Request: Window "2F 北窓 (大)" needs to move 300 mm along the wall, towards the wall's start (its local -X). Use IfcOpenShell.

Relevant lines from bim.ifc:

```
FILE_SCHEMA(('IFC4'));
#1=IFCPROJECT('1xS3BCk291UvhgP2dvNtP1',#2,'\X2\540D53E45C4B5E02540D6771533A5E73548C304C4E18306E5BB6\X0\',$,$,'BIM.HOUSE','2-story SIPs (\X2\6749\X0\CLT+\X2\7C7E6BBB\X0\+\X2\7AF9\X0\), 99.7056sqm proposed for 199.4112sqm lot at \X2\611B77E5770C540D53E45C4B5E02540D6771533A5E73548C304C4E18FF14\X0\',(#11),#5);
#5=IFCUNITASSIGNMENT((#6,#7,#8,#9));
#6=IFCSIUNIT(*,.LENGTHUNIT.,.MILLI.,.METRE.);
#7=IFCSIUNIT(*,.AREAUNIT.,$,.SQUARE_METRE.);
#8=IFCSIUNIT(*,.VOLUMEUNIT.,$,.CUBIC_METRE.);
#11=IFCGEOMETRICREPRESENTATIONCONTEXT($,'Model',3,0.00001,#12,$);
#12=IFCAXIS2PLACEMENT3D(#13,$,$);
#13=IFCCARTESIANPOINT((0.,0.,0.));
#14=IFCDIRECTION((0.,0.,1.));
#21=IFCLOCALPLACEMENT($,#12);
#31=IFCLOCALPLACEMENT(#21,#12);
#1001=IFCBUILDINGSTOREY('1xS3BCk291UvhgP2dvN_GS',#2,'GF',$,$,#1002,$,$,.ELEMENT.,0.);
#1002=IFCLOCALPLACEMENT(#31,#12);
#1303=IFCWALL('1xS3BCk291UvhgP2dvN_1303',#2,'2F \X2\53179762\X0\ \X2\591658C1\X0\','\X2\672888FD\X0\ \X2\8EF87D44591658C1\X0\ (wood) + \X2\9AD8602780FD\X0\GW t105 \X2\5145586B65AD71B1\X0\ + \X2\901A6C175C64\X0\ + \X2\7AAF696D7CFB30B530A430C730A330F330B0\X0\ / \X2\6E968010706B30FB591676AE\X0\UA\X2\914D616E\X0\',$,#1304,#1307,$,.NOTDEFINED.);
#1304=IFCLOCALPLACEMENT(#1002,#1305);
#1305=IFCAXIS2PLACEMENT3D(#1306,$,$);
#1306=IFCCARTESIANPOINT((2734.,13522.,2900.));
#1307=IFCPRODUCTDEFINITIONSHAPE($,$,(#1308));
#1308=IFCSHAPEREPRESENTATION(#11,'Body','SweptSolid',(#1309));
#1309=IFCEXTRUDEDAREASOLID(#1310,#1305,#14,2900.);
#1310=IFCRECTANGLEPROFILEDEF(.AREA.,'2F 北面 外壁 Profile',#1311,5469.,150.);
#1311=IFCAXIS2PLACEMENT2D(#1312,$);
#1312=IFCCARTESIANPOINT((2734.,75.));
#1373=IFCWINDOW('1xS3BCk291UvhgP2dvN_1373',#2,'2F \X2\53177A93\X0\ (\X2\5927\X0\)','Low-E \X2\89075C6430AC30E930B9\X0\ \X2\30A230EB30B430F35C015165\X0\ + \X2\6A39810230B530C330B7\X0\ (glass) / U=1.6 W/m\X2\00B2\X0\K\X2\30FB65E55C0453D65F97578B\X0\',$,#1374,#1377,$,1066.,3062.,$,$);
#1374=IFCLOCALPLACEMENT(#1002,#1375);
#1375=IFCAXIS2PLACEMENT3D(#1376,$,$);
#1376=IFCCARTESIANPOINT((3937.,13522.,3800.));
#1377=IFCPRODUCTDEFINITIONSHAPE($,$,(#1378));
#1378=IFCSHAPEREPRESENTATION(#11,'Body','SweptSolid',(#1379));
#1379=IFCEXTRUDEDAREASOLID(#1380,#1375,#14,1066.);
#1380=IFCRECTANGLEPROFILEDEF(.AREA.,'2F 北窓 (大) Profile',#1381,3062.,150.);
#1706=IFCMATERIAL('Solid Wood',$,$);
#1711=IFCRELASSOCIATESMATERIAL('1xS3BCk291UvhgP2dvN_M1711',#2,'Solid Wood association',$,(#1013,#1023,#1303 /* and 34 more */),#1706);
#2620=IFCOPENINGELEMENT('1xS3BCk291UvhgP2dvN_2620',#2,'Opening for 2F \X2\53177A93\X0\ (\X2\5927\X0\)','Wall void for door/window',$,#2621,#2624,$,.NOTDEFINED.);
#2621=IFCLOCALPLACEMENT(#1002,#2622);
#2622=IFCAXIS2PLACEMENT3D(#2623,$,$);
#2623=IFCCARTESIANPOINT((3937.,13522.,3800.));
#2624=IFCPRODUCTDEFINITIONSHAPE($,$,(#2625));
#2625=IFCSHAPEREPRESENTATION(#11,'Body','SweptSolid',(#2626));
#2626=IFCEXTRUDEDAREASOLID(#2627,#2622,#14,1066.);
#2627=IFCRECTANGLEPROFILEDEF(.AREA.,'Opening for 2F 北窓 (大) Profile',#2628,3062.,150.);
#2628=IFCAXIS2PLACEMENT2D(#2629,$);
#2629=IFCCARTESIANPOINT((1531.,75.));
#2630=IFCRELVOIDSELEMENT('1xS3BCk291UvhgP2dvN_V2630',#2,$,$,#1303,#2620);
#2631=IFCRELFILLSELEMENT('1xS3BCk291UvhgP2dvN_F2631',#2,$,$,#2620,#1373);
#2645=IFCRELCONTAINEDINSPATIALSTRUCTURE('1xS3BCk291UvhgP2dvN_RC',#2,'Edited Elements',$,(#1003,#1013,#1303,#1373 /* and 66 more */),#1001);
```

```python
import ifcopenshell
import ifcopenshell.api.geometry
import ifcopenshell.util.placement

model = ifcopenshell.open("bim.ifc")

window = model.by_id(1373)
opening = window.FillsVoids[0].RelatingOpeningElement
wall = opening.VoidsElements[0].RelatingBuildingElement

wall_matrix = ifcopenshell.util.placement.get_local_placement(wall.ObjectPlacement)
shift = wall_matrix[:3, 0] * -300.0
before = ifcopenshell.util.placement.get_local_placement(window.ObjectPlacement)[:3, 3].copy()

# The window is not placed relative to its opening, so move both.
for product in (opening, window):
    matrix = ifcopenshell.util.placement.get_local_placement(product.ObjectPlacement)
    matrix[:3, 3] += shift
    ifcopenshell.api.geometry.edit_object_placement(model, product=product, matrix=matrix, is_si=False)

after = ifcopenshell.util.placement.get_local_placement(window.ObjectPlacement)[:3, 3]
print("window moved by", (after - before).round(3) + 0.0)

model.write("bim-out.ifc")
```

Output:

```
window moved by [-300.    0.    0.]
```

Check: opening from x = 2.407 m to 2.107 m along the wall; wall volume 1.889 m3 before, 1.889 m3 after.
